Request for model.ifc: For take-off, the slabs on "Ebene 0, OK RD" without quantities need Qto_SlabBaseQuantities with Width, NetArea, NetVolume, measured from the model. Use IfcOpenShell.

First a look at what the model holds.

```python
import ifcopenshell
import ifcopenshell.util.element
import ifcopenshell.util.unit

model = ifcopenshell.open("model.ifc")
print(model.schema)
for unit_type in ("LENGTHUNIT", "AREAUNIT", "VOLUMEUNIT"):
    print(unit_type, ifcopenshell.util.unit.calculate_unit_scale(model, unit_type))
storey = next(s for s in model.by_type("IfcBuildingStorey") if s.Name == "Ebene 0, OK RD")
slabs = [e for e in ifcopenshell.util.element.get_decomposition(storey) if e.is_a("IfcSlab")]
for e in sorted(slabs, key=lambda e: e.id()):
    print(e.id(), e.is_a(), e.Name, list(ifcopenshell.util.element.get_psets(e, qtos_only=True)), sep=" | ")
```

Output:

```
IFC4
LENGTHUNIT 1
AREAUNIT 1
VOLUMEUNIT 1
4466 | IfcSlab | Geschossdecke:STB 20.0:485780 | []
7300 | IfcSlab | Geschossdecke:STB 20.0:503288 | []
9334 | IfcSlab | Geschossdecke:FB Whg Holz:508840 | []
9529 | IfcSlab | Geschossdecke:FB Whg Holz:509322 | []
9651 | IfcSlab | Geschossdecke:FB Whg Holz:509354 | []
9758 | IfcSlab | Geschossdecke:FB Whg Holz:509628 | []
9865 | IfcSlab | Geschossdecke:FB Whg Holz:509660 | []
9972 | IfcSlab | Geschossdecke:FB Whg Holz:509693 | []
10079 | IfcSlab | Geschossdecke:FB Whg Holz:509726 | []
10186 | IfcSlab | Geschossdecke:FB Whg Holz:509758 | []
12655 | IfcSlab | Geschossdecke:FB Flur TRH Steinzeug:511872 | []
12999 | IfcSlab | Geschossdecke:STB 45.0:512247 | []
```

```python
import ifcopenshell
import ifcopenshell.api.pset
import ifcopenshell.geom
import ifcopenshell.util.element
import ifcopenshell.util.shape
import ifcopenshell.util.unit

model = ifcopenshell.open("model.ifc")
unit_scale = ifcopenshell.util.unit.calculate_unit_scale(model)
area_scale = ifcopenshell.util.unit.calculate_unit_scale(model, "AREAUNIT")
volume_scale = ifcopenshell.util.unit.calculate_unit_scale(model, "VOLUMEUNIT")
settings = ifcopenshell.geom.settings()

storey = next(s for s in model.by_type("IfcBuildingStorey") if s.Name == "Ebene 0, OK RD")
slabs = [e for e in ifcopenshell.util.element.get_decomposition(storey) if e.is_a("IfcSlab")]

for e in sorted(slabs, key=lambda e: e.id()):
    if ifcopenshell.util.element.get_psets(e, qtos_only=True, should_inherit=False):
        continue
    # Geometry comes back in metres, in the element's own axes.
    shape = ifcopenshell.geom.create_shape(settings, e)
    values = {
        "Width": ifcopenshell.util.shape.get_z(shape.geometry) / unit_scale,
        "NetArea": ifcopenshell.util.shape.get_footprint_area(shape.geometry) / area_scale,
        "NetVolume": ifcopenshell.util.shape.get_volume(shape.geometry) / volume_scale,
    }
    qto = ifcopenshell.api.pset.add_qto(model, product=e, name="Qto_SlabBaseQuantities")
    ifcopenshell.api.pset.edit_qto(model, qto=qto, properties=values)
    print(e.id(), {k: round(v, 3) for k, v in values.items()})

model.write("model_edited.ifc")
```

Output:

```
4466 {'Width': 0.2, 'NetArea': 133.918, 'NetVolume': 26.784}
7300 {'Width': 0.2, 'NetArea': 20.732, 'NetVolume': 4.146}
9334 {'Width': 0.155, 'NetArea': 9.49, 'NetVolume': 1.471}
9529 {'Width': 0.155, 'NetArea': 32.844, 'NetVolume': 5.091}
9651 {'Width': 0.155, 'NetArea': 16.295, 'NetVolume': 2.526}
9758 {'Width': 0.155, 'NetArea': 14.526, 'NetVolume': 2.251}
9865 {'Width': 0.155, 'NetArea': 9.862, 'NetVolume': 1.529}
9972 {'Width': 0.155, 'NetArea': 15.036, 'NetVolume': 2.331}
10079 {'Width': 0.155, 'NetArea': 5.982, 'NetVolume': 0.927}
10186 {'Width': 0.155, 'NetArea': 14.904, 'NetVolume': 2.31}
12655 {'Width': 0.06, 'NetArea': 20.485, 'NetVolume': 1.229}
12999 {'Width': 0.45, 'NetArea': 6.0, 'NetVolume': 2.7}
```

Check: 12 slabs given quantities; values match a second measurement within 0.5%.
